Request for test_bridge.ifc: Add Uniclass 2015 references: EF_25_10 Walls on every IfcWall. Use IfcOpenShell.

First a look at what the model holds.

```python
import ifcopenshell

model = ifcopenshell.open("test_bridge.ifc")
print(model.schema)
print("classifications:", [c.Name for c in model.by_type("IfcClassification")])
for ifc_class in ("IfcDoor", "IfcRoof", "IfcStair", "IfcWall", "IfcWindow"):
    print(ifc_class, len(model.by_type(ifc_class)))
```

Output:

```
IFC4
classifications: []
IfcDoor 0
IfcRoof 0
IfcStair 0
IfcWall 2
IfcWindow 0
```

```python
import ifcopenshell
import ifcopenshell.api.classification

model = ifcopenshell.open("test_bridge.ifc")

system = ifcopenshell.api.classification.add_classification(model, classification="Uniclass 2015")

codes = {
    "IfcWall": ("EF_25_10", "Walls"),
}
for ifc_class, (code, name) in codes.items():
    products = model.by_type(ifc_class)
    ifcopenshell.api.classification.add_reference(
        model, products=products, classification=system, identification=code, name=name
    )
    print(code, len(products))

model.write("test_bridge_rev.ifc")
```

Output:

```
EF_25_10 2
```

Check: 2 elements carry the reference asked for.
